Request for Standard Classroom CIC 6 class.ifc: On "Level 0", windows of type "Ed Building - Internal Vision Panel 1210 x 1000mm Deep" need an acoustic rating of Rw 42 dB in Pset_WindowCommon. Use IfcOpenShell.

First a look at what the model holds.

```python
import ifcopenshell
import ifcopenshell.util.element

model = ifcopenshell.open("Standard Classroom CIC 6 class.ifc")
print(model.schema)
storey = next(s for s in model.by_type("IfcBuildingStorey") if s.Name == "Level 0")
windows = [e for e in ifcopenshell.util.element.get_decomposition(storey) if e.is_a("IfcWindow")]
seen = {}
for e in windows:
    element_type = ifcopenshell.util.element.get_type(e)
    key = (element_type.Name if element_type != e and element_type else None, ifcopenshell.util.element.get_pset(e, "Pset_WindowCommon", "AcousticRating"))
    seen[key] = seen.get(key, 0) + 1
for (name, value), count in sorted(seen.items(), key=str):
    print(count, "x", name, "|", value)
```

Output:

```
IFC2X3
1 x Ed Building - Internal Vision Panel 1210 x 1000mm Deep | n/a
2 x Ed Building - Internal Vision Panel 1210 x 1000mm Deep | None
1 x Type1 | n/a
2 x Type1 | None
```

```python
import ifcopenshell
import ifcopenshell.api.pset
import ifcopenshell.util.element

model = ifcopenshell.open("Standard Classroom CIC 6 class.ifc")

storey = next(s for s in model.by_type("IfcBuildingStorey") if s.Name == "Level 0")
windows = [e for e in ifcopenshell.util.element.get_decomposition(storey) if e.is_a("IfcWindow")]

count = 0
for e in windows:
    element_type = ifcopenshell.util.element.get_type(e)
    if element_type in (None, e) or element_type.Name != "Ed Building - Internal Vision Panel 1210 x 1000mm Deep":
        continue
    # add_pset returns the element's existing set when there is one.
    pset = ifcopenshell.api.pset.add_pset(model, product=e, name="Pset_WindowCommon")
    ifcopenshell.api.pset.edit_pset(model, pset=pset, properties={"AcousticRating": "Rw 42 dB"})
    count += 1

print(count, "windows updated")

model.write("Standard Classroom CIC 6 class_v2.ifc")
```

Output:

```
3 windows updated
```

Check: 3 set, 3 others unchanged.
